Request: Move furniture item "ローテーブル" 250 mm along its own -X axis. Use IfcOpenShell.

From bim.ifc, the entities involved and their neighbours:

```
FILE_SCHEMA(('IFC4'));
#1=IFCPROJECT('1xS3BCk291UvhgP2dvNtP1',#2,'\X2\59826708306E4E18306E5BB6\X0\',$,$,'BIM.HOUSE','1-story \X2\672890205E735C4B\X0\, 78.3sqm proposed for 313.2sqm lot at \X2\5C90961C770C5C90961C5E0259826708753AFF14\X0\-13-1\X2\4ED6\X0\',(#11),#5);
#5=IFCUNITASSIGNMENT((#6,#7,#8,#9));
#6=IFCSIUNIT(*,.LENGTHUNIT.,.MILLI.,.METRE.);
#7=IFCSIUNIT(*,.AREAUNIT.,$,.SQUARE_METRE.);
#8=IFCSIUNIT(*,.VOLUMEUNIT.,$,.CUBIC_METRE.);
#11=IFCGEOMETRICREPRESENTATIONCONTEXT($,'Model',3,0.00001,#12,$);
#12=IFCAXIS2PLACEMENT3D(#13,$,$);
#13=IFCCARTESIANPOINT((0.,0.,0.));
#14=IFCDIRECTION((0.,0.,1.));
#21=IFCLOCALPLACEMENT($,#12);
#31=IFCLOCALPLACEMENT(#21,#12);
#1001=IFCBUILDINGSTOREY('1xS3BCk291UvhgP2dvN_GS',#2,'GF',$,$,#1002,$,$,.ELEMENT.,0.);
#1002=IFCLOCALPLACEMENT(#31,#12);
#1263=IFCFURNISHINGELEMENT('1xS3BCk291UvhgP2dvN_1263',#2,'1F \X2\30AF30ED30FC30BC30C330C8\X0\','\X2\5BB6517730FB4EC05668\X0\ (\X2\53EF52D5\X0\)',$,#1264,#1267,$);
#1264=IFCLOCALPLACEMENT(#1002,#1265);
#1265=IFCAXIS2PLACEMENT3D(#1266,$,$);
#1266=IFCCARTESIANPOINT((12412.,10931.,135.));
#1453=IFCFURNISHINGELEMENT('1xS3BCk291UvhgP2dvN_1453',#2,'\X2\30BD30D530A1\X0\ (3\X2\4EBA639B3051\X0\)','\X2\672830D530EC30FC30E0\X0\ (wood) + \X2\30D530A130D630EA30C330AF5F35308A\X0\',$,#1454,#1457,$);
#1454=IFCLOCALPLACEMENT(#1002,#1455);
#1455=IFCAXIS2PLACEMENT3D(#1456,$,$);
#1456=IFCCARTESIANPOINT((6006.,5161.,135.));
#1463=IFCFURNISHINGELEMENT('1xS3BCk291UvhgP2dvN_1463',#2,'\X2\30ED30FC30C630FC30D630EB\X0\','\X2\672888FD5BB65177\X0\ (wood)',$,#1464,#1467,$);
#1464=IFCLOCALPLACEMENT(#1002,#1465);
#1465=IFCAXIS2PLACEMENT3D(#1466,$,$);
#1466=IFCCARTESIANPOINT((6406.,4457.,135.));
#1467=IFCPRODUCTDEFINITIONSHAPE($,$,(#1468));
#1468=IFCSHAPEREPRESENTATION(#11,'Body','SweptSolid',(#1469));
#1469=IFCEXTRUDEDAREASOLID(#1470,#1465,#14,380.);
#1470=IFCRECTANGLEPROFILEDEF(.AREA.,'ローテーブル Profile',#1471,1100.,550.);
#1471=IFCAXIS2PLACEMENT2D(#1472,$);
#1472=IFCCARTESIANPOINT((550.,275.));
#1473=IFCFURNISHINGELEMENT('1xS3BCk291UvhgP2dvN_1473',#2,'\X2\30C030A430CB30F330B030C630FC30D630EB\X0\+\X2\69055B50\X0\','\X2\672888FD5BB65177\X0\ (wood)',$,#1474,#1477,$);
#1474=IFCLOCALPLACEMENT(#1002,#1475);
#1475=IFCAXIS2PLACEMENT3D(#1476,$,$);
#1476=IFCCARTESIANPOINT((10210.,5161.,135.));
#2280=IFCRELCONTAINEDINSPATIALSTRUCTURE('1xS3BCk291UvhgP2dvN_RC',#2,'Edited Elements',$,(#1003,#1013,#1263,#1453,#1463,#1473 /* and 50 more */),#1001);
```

```python
import ifcopenshell
import ifcopenshell.api.geometry
import ifcopenshell.util.placement
import ifcopenshell.util.unit

model = ifcopenshell.open("bim.ifc")
unit_scale = ifcopenshell.util.unit.calculate_unit_scale(model)

item = model.by_id(1463)
matrix = ifcopenshell.util.placement.get_local_placement(item.ObjectPlacement)
matrix[:3, 3] -= matrix[:3, 0] * 0.25 / unit_scale
ifcopenshell.api.geometry.edit_object_placement(model, product=item, matrix=matrix, is_si=False)

print(ifcopenshell.util.placement.get_local_placement(item.ObjectPlacement).round(3) + 0.0)

model.write("bim_updated.ifc")
```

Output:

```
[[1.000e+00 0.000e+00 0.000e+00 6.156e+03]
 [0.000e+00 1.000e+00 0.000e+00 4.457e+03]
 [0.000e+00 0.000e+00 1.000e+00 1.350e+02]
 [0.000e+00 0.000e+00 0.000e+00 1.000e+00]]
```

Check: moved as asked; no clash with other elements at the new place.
